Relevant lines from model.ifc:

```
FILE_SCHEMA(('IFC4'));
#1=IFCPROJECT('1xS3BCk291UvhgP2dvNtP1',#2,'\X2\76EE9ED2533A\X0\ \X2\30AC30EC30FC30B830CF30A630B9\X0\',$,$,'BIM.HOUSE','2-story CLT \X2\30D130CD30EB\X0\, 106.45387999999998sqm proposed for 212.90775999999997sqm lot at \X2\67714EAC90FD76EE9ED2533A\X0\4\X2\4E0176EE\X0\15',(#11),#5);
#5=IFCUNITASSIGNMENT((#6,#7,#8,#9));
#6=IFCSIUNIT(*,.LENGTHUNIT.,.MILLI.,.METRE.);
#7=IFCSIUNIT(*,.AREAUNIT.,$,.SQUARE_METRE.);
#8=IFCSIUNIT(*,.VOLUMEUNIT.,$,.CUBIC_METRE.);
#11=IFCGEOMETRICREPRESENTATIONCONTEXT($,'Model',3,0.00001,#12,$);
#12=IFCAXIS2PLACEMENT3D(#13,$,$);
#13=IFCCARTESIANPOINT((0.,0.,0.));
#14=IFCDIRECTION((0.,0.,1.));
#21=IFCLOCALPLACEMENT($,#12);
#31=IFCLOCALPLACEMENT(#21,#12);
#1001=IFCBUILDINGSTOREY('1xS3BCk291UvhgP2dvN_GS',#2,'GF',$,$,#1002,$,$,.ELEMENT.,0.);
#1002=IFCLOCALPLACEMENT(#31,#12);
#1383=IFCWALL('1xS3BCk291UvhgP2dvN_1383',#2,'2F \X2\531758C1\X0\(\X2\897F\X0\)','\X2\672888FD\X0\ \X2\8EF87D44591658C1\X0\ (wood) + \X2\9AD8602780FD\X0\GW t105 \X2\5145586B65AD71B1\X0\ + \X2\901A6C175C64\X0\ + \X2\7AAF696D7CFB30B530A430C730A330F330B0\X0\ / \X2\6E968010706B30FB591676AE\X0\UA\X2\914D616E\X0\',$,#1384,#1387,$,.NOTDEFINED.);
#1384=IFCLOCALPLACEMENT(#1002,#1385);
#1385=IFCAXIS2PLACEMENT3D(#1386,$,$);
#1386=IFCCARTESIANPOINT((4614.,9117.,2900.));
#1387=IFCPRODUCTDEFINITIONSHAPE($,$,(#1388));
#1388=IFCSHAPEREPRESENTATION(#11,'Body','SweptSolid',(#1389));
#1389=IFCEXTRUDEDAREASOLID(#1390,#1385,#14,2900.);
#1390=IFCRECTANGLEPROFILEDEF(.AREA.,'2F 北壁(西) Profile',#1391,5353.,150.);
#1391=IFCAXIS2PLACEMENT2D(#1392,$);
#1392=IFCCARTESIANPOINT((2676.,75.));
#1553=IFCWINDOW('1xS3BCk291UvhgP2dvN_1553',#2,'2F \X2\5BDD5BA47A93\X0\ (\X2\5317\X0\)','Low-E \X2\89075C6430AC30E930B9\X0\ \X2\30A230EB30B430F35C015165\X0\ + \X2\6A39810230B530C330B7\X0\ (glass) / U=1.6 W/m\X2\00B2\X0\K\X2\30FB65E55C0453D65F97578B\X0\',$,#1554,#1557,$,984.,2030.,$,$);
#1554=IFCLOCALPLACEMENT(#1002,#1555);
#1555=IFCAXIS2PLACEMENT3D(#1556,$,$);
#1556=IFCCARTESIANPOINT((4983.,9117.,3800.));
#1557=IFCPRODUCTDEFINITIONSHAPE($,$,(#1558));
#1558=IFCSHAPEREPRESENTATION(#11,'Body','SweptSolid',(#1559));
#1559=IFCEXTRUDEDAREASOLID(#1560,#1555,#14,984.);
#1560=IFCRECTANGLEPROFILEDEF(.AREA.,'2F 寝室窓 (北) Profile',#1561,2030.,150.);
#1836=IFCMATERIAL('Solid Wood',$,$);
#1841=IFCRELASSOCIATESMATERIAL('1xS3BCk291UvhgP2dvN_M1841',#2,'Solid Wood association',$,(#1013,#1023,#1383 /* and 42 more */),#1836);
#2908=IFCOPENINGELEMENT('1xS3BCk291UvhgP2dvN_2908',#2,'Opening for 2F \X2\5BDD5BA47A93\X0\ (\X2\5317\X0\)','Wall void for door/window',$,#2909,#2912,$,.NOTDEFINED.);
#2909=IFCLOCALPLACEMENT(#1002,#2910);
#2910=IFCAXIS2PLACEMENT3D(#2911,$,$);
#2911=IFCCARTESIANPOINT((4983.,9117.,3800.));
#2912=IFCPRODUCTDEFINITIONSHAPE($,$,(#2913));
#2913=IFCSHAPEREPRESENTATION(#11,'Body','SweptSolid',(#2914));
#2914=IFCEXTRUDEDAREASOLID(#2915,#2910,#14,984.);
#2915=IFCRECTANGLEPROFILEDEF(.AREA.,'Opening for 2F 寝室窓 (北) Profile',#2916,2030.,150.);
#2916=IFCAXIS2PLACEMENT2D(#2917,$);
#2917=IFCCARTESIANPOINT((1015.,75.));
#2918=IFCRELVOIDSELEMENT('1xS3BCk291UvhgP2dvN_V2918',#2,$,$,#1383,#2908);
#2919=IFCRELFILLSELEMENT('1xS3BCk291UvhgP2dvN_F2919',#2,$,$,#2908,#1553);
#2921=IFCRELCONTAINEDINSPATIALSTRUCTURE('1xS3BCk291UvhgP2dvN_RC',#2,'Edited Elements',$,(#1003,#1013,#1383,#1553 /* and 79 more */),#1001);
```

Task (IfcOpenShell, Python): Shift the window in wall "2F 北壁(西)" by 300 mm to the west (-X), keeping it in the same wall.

```python
import ifcopenshell
import ifcopenshell.api.geometry
import ifcopenshell.util.placement
import ifcopenshell.util.unit

model = ifcopenshell.open("model.ifc")
unit_scale = ifcopenshell.util.unit.calculate_unit_scale(model)

window = model.by_guid("1xS3BCk291UvhgP2dvN_1553")
opening = window.FillsVoids[0].RelatingOpeningElement
wall = opening.VoidsElements[0].RelatingBuildingElement

wall_matrix = ifcopenshell.util.placement.get_local_placement(wall.ObjectPlacement)
shift = wall_matrix[:3, 0] * -0.3 / unit_scale
before = ifcopenshell.util.placement.get_local_placement(window.ObjectPlacement)[:3, 3].copy()

# The window is not placed relative to its opening, so move both.
for product in (opening, window):
    matrix = ifcopenshell.util.placement.get_local_placement(product.ObjectPlacement)
    matrix[:3, 3] += shift
    ifcopenshell.api.geometry.edit_object_placement(model, product=product, matrix=matrix, is_si=False)

after = ifcopenshell.util.placement.get_local_placement(window.ObjectPlacement)[:3, 3]
print("window moved by", (after - before).round(3) + 0.0)

model.write("model_updated.ifc")
```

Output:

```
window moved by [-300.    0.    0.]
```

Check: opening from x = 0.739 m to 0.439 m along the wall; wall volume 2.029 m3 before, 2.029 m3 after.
